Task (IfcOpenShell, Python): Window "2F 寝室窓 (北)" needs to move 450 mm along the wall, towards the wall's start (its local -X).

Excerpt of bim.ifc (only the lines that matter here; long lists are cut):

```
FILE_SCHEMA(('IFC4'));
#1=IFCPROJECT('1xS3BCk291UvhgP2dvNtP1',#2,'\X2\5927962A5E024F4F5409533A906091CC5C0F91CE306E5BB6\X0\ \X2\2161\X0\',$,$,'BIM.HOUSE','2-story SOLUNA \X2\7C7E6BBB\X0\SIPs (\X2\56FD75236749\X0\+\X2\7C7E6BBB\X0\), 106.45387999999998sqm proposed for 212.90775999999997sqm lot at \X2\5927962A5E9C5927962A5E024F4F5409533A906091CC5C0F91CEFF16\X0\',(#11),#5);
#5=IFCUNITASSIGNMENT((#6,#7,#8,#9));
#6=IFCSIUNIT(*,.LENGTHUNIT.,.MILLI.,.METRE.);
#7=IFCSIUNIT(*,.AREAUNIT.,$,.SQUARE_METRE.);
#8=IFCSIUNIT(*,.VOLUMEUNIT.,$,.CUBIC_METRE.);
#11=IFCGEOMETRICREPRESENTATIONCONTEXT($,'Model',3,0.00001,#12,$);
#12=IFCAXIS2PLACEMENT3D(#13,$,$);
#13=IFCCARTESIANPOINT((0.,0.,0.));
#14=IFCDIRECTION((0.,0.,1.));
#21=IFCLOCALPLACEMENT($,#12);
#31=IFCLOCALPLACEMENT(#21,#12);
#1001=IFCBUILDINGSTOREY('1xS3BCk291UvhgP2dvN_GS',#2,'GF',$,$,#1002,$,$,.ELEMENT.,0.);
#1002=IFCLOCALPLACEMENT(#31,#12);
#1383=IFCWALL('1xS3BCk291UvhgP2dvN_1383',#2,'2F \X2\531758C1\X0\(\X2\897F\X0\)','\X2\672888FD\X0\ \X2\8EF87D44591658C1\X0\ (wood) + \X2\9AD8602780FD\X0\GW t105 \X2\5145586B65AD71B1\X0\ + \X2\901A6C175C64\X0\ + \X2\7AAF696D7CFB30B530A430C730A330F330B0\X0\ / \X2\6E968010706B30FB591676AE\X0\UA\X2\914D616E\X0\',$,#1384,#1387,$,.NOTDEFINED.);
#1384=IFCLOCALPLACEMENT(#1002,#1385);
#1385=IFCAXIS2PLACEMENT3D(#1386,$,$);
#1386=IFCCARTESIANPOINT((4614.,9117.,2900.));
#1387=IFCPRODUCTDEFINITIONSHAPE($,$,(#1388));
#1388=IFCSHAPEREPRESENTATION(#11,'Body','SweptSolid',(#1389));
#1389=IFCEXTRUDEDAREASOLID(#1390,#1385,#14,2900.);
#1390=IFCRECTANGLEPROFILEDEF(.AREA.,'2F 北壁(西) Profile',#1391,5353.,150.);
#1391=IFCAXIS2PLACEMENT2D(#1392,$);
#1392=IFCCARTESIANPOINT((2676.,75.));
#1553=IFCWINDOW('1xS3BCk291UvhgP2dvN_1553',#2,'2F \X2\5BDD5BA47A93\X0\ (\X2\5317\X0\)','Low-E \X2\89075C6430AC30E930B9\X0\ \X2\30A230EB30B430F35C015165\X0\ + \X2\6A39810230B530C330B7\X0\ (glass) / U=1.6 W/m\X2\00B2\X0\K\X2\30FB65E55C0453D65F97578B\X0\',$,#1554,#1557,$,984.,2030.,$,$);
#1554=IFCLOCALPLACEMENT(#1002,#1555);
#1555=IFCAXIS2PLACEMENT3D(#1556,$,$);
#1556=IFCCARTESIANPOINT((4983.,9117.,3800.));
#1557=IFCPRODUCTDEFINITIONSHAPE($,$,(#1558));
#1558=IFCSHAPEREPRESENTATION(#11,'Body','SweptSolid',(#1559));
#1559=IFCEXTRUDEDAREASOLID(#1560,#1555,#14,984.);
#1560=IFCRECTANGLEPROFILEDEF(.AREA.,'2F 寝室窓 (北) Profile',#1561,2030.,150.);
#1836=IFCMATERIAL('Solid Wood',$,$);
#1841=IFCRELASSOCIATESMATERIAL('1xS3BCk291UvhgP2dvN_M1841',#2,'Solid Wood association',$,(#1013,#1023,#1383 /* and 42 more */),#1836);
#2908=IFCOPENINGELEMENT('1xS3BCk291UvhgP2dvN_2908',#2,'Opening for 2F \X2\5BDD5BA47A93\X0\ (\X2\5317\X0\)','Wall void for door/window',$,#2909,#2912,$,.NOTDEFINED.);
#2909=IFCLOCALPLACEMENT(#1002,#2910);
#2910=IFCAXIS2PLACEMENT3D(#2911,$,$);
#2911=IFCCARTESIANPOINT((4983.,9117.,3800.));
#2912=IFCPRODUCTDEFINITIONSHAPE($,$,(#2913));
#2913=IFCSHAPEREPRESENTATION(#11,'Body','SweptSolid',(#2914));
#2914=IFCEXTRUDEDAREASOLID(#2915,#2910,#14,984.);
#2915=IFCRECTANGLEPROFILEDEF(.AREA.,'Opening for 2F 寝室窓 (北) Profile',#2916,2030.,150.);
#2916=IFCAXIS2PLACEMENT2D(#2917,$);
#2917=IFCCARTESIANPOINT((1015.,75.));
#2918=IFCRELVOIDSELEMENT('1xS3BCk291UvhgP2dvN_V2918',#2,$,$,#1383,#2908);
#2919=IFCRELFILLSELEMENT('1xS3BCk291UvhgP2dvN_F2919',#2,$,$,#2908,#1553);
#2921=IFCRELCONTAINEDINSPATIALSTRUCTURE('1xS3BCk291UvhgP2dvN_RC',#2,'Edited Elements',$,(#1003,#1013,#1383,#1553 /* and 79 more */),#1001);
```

```python
import ifcopenshell
import ifcopenshell.api.geometry
import ifcopenshell.util.placement
import ifcopenshell.util.unit

model = ifcopenshell.open("bim.ifc")
unit_scale = ifcopenshell.util.unit.calculate_unit_scale(model)

window = model.by_guid("1xS3BCk291UvhgP2dvN_1553")
opening = window.FillsVoids[0].RelatingOpeningElement
wall = opening.VoidsElements[0].RelatingBuildingElement

wall_matrix = ifcopenshell.util.placement.get_local_placement(wall.ObjectPlacement)
shift = wall_matrix[:3, 0] * -0.45 / unit_scale
before = ifcopenshell.util.placement.get_local_placement(window.ObjectPlacement)[:3, 3].copy()

# The window is not placed relative to its opening, so move both.
for product in (opening, window):
    matrix = ifcopenshell.util.placement.get_local_placement(product.ObjectPlacement)
    matrix[:3, 3] += shift
    ifcopenshell.api.geometry.edit_object_placement(model, product=product, matrix=matrix, is_si=False)

after = ifcopenshell.util.placement.get_local_placement(window.ObjectPlacement)[:3, 3]
print("window moved by", (after - before).round(3) + 0.0)

model.write("bim_updated.ifc")
```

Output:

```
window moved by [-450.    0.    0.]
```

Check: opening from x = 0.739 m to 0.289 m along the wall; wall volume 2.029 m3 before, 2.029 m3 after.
